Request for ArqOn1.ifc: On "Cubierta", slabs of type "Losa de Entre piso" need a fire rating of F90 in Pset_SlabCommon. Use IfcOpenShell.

First a look at what the model holds.

```python
import ifcopenshell
import ifcopenshell.util.element

model = ifcopenshell.open("ArqOn1.ifc")
print(model.schema)
storey = next(s for s in model.by_type("IfcBuildingStorey") if s.Name == "Cubierta")
slabs = [e for e in ifcopenshell.util.element.get_decomposition(storey) if e.is_a("IfcSlab")]
seen = {}
for e in slabs:
    element_type = ifcopenshell.util.element.get_type(e)
    key = (element_type.Name if element_type != e and element_type else None, ifcopenshell.util.element.get_pset(e, "Pset_SlabCommon", "FireRating"))
    seen[key] = seen.get(key, 0) + 1
for (name, value), count in sorted(seen.items(), key=str):
    print(count, "x", name, "|", value)
```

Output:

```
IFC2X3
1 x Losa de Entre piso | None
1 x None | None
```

```python
import ifcopenshell
import ifcopenshell.api.pset
import ifcopenshell.util.element

model = ifcopenshell.open("ArqOn1.ifc")

storey = next(s for s in model.by_type("IfcBuildingStorey") if s.Name == "Cubierta")
slabs = [e for e in ifcopenshell.util.element.get_decomposition(storey) if e.is_a("IfcSlab")]

count = 0
for e in slabs:
    element_type = ifcopenshell.util.element.get_type(e)
    if element_type in (None, e) or element_type.Name != "Losa de Entre piso":
        continue
    # add_pset returns the element's existing set when there is one.
    pset = ifcopenshell.api.pset.add_pset(model, product=e, name="Pset_SlabCommon")
    ifcopenshell.api.pset.edit_pset(model, pset=pset, properties={"FireRating": "F90"})
    count += 1

print(count, "slabs updated")

model.write("ArqOn1_updated.ifc")
```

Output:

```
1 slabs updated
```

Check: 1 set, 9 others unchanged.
